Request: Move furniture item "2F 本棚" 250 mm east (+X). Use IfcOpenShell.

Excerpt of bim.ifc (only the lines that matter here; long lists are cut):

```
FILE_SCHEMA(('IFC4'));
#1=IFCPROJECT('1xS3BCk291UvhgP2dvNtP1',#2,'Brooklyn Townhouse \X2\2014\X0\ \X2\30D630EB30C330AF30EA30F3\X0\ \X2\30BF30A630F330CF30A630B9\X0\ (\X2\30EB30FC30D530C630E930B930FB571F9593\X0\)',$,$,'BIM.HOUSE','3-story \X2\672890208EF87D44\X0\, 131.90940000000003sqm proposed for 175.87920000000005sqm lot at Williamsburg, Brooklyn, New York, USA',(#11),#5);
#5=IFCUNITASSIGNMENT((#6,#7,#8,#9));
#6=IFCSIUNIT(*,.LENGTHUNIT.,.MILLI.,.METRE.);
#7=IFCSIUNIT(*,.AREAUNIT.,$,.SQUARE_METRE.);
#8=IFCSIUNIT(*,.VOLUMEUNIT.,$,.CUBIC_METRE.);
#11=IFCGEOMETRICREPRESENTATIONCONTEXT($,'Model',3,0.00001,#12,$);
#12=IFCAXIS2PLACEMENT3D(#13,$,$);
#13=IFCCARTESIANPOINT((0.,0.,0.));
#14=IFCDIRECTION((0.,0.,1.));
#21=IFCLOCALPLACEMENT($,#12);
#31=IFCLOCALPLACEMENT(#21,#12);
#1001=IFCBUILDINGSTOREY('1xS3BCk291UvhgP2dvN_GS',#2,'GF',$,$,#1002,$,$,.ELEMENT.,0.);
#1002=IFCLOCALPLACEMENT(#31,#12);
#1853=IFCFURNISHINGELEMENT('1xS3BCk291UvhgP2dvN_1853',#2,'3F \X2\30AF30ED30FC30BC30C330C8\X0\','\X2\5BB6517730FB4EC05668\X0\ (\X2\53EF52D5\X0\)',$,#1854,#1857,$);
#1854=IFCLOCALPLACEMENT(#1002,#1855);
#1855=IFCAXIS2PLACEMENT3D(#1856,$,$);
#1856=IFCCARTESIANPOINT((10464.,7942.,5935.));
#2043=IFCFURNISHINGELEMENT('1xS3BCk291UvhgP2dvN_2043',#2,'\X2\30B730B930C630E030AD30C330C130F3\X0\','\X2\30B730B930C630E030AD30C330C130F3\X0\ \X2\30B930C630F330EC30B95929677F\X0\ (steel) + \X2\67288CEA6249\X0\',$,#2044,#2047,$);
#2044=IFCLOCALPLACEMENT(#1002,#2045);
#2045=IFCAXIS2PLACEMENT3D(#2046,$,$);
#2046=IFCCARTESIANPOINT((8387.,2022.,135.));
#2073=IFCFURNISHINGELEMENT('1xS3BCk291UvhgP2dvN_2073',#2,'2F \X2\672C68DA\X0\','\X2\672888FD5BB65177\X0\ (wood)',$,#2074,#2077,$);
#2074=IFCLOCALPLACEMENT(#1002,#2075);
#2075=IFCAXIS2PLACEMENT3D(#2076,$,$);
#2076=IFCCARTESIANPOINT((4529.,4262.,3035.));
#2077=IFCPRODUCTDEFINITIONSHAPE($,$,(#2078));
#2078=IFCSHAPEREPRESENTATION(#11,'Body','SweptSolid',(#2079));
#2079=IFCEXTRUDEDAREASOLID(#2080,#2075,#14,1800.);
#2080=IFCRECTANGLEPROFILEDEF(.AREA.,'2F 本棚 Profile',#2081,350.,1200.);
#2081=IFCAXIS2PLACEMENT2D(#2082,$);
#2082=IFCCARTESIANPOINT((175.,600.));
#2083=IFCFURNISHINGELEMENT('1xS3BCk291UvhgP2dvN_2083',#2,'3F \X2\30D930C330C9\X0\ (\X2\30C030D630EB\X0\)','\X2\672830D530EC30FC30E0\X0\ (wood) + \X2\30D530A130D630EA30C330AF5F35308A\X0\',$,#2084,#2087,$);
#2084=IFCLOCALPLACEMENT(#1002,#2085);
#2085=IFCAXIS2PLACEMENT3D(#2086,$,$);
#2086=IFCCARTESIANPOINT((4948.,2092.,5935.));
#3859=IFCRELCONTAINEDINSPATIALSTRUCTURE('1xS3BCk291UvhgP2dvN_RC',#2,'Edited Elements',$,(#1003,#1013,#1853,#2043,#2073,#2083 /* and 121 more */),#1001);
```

```python
import ifcopenshell
import ifcopenshell.api.geometry
import ifcopenshell.util.placement

model = ifcopenshell.open("bim.ifc")

item = model.by_guid("1xS3BCk291UvhgP2dvN_2073")
matrix = ifcopenshell.util.placement.get_local_placement(item.ObjectPlacement)
matrix[0, 3] += 250.0
ifcopenshell.api.geometry.edit_object_placement(model, product=item, matrix=matrix, is_si=False)

print(ifcopenshell.util.placement.get_local_placement(item.ObjectPlacement).round(3) + 0.0)

model.write("bim_v2.ifc")
```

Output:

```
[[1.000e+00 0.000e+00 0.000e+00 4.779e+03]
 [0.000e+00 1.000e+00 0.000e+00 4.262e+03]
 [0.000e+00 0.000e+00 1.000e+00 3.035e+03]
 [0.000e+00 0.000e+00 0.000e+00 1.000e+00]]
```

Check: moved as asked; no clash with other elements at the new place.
